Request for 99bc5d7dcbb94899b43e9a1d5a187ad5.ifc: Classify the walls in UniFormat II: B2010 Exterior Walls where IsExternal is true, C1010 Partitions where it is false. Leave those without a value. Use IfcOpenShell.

First a look at what the model holds.

```python
import ifcopenshell
import ifcopenshell.util.element

model = ifcopenshell.open("99bc5d7dcbb94899b43e9a1d5a187ad5.ifc")
print(model.schema)
print("classifications:", [c.Name for c in model.by_type("IfcClassification")])
values = [ifcopenshell.util.element.get_pset(e, "Pset_WallCommon", "IsExternal") for e in model.by_type("IfcWall")]
for value in (True, False, None):
    print("IsExternal", value, values.count(value))
```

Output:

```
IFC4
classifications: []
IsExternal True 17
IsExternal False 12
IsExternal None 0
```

```python
import ifcopenshell
import ifcopenshell.api.classification
import ifcopenshell.util.element

model = ifcopenshell.open("99bc5d7dcbb94899b43e9a1d5a187ad5.ifc")

system = ifcopenshell.api.classification.add_classification(model, classification="UniFormat II")

walls = model.by_type("IfcWall")
external = {e: ifcopenshell.util.element.get_pset(e, "Pset_WallCommon", "IsExternal") for e in walls}
for flag, code, name in ((True, "B2010", "Exterior Walls"), (False, "C1010", "Partitions")):
    products = [e for e in walls if external[e] is flag]
    ifcopenshell.api.classification.add_reference(
        model, products=products, classification=system, identification=code, name=name
    )
    print(code, len(products))

model.write("99bc5d7dcbb94899b43e9a1d5a187ad5_edited.ifc")
```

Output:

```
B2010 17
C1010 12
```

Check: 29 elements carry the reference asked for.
